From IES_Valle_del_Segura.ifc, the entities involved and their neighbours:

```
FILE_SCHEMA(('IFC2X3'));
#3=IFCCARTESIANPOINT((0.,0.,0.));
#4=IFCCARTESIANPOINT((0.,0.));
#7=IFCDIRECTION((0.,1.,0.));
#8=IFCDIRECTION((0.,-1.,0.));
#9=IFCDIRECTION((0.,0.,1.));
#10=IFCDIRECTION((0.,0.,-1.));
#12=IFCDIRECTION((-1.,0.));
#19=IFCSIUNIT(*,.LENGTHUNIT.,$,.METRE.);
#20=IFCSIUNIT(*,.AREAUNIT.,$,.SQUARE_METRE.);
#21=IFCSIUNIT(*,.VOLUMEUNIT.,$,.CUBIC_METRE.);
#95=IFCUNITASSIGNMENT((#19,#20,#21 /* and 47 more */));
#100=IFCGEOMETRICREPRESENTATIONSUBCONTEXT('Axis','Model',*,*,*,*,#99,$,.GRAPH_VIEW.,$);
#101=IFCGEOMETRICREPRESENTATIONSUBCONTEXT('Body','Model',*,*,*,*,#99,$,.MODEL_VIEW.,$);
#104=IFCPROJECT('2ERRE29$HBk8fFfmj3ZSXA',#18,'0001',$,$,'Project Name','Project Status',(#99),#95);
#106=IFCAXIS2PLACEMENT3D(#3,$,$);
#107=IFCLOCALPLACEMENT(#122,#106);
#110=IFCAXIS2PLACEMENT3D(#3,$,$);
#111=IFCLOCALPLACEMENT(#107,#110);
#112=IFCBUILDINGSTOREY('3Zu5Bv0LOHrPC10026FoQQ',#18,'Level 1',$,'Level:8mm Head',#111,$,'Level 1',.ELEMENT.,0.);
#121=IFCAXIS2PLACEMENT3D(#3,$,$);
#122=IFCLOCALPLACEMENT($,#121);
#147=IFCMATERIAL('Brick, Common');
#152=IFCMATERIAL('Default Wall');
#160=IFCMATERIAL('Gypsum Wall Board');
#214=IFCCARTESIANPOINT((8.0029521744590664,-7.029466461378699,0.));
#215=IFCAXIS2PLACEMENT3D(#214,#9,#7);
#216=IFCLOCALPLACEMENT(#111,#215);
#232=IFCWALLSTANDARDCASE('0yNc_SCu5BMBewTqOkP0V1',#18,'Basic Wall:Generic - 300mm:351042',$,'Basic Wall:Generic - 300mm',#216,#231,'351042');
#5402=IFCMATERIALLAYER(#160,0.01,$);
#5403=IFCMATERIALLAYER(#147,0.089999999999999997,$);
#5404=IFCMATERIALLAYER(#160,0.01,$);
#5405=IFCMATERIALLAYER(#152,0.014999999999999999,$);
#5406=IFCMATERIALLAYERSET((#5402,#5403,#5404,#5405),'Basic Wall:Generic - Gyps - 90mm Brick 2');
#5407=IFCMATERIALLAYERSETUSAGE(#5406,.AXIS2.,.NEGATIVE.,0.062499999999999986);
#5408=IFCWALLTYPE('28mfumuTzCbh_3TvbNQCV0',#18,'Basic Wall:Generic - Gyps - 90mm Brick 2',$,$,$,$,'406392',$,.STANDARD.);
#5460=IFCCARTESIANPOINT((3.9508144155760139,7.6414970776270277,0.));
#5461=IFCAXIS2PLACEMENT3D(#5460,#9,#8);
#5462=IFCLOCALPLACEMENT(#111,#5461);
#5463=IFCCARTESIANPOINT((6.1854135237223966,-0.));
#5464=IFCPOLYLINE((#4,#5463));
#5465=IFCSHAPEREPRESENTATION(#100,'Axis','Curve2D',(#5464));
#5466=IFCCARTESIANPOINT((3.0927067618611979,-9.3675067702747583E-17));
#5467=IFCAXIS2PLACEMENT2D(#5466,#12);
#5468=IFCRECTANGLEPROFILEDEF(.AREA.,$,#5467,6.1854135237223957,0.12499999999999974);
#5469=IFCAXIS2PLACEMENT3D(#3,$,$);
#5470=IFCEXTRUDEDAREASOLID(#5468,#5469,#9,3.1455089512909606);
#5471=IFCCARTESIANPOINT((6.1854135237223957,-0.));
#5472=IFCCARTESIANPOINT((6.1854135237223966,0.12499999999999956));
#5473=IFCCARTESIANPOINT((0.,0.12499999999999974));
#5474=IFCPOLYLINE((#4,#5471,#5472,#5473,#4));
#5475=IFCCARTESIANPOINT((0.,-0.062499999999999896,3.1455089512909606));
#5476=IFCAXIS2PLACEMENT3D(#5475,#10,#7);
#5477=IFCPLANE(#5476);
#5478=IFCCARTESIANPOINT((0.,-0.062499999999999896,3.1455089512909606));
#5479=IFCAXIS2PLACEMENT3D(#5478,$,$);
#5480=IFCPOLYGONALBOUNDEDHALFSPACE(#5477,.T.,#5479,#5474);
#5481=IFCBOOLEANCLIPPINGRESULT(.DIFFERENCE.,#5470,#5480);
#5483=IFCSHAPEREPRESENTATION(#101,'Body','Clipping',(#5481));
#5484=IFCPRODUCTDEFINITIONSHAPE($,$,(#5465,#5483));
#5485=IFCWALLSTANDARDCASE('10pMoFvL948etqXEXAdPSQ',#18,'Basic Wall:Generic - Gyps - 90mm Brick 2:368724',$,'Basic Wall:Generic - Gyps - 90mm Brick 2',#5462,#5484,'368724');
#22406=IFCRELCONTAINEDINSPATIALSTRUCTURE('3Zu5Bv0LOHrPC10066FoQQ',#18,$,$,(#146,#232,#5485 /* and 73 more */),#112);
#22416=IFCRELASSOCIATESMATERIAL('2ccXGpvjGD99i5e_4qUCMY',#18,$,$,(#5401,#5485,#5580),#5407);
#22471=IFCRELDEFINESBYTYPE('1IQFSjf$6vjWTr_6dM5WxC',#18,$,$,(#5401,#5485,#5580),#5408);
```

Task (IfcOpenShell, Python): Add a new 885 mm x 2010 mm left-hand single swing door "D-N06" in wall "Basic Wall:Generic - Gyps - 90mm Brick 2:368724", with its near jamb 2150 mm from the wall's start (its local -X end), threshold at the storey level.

```python
import numpy as np
import ifcopenshell
import ifcopenshell.api.feature
import ifcopenshell.api.geometry
import ifcopenshell.api.root
import ifcopenshell.api.spatial
import ifcopenshell.api.type
import ifcopenshell.geom
import ifcopenshell.util.element
import ifcopenshell.util.placement
import ifcopenshell.util.representation
import ifcopenshell.util.shape
import ifcopenshell.util.unit

model = ifcopenshell.open("IES_Valle_del_Segura.ifc")
unit_scale = ifcopenshell.util.unit.calculate_unit_scale(model)
settings = ifcopenshell.geom.settings()


def volume(element):
    """Net volume in cubic metres, openings subtracted."""
    shape = ifcopenshell.geom.create_shape(settings, element)
    return ifcopenshell.util.shape.get_volume(shape.geometry)


wall = model.by_guid("10pMoFvL948etqXEXAdPSQ")
storey = ifcopenshell.util.element.get_container(wall, ifc_class="IfcBuildingStorey")
context = ifcopenshell.util.representation.get_context(model, "Model", "Body", "MODEL_VIEW")
before = volume(wall)

width, height, from_end, sill = 0.885, 2.01, 2.15, 0.0  # metres

# The wall runs along its own X axis, and the end named is its -X end.
wall_shape = ifcopenshell.geom.create_shape(settings, wall)
x, y, z = ifcopenshell.util.shape.get_vertices(wall_shape.geometry).T
start = x.min() + from_end
face, thickness = float(y.min()), float(y.max() - y.min())
wall_matrix = ifcopenshell.util.placement.get_local_placement(wall.ObjectPlacement)
level = ifcopenshell.util.placement.get_local_placement(storey.ObjectPlacement)[2, 3]


def in_wall(x, y):
    """Placement at x, y metres in the wall's axes, at sill height."""
    matrix = wall_matrix.copy()
    matrix[:, 3] = wall_matrix @ np.array([x / unit_scale, y / unit_scale, 0.0, 1.0])
    matrix[2, 3] = level + sill / unit_scale
    return matrix


# Opening: a box that overshoots both wall faces by 50 mm.
opening = ifcopenshell.api.root.create_entity(model, ifc_class="IfcOpeningElement")
box = ifcopenshell.api.geometry.add_wall_representation(
    model, context=context, length=width, height=height, thickness=thickness + 0.1
)
ifcopenshell.api.geometry.assign_representation(model, product=opening, representation=box)
ifcopenshell.api.geometry.edit_object_placement(model, product=opening, matrix=in_wall(start, face - 0.05), is_si=False)
ifcopenshell.api.feature.add_feature(model, feature=opening, element=wall)

door = ifcopenshell.api.root.create_entity(model, ifc_class="IfcDoor", name="D-N06")
door.OverallWidth, door.OverallHeight = width / unit_scale, height / unit_scale
body = ifcopenshell.api.geometry.add_door_representation(
    model,
    context=context,
    overall_width=door.OverallWidth,
    overall_height=door.OverallHeight,
    operation_type="SINGLE_SWING_LEFT",
    lining_properties={"LiningDepth": thickness / unit_scale, "ThresholdDepth": thickness / unit_scale},
)
ifcopenshell.api.geometry.assign_representation(model, product=door, representation=body)
ifcopenshell.api.spatial.assign_container(model, products=[door], relating_structure=storey)
fills = ifcopenshell.api.feature.add_filling(model, opening=opening, element=door)
fills.OwnerHistory = door.OwnerHistory  # required in IFC2X3

# IFC2X3 keeps the operation on the door style.
style = ifcopenshell.api.root.create_entity(model, ifc_class="IfcDoorStyle", name="D-N06")
style.OperationType, style.ConstructionType = "SINGLE_SWING_LEFT", "NOTDEFINED"
style.ParameterTakesPrecedence = style.Sizeable = False
ifcopenshell.api.type.assign_type(model, related_objects=[door], relating_type=style)

# The lining spans the wall, so the door starts at the wall face.
ifcopenshell.api.geometry.edit_object_placement(model, product=door, matrix=in_wall(start, face), is_si=False)

after = volume(wall)

print(f"wall volume {before:.3f} -> {after:.3f} m3")

model.write("IES_Valle_del_Segura_edited.ifc")
```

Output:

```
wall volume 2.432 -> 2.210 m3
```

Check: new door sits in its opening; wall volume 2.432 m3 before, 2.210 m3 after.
